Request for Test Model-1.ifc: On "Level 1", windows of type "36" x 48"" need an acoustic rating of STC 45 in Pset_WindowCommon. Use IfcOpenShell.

First a look at what the model holds.

```python
import ifcopenshell
import ifcopenshell.util.element

model = ifcopenshell.open("Test Model-1.ifc")
print(model.schema)
storey = next(s for s in model.by_type("IfcBuildingStorey") if s.Name == "Level 1")
windows = [e for e in ifcopenshell.util.element.get_decomposition(storey) if e.is_a("IfcWindow")]
seen = {}
for e in windows:
    element_type = ifcopenshell.util.element.get_type(e)
    key = (element_type.Name if element_type != e and element_type else None, ifcopenshell.util.element.get_pset(e, "Pset_WindowCommon", "AcousticRating"))
    seen[key] = seen.get(key, 0) + 1
for (name, value), count in sorted(seen.items(), key=str):
    print(count, "x", name, "|", value)
```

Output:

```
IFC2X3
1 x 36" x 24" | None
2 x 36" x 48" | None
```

```python
import ifcopenshell
import ifcopenshell.api.pset
import ifcopenshell.util.element

model = ifcopenshell.open("Test Model-1.ifc")

storey = next(s for s in model.by_type("IfcBuildingStorey") if s.Name == "Level 1")
windows = [e for e in ifcopenshell.util.element.get_decomposition(storey) if e.is_a("IfcWindow")]

count = 0
for e in windows:
    element_type = ifcopenshell.util.element.get_type(e)
    if element_type in (None, e) or element_type.Name != '36" x 48"':
        continue
    # add_pset returns the element's existing set when there is one.
    pset = ifcopenshell.api.pset.add_pset(model, product=e, name="Pset_WindowCommon")
    ifcopenshell.api.pset.edit_pset(model, pset=pset, properties={"AcousticRating": "STC 45"})
    count += 1

print(count, "windows updated")

model.write("Test Model-1_edited.ifc")
```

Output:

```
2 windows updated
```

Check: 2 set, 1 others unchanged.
